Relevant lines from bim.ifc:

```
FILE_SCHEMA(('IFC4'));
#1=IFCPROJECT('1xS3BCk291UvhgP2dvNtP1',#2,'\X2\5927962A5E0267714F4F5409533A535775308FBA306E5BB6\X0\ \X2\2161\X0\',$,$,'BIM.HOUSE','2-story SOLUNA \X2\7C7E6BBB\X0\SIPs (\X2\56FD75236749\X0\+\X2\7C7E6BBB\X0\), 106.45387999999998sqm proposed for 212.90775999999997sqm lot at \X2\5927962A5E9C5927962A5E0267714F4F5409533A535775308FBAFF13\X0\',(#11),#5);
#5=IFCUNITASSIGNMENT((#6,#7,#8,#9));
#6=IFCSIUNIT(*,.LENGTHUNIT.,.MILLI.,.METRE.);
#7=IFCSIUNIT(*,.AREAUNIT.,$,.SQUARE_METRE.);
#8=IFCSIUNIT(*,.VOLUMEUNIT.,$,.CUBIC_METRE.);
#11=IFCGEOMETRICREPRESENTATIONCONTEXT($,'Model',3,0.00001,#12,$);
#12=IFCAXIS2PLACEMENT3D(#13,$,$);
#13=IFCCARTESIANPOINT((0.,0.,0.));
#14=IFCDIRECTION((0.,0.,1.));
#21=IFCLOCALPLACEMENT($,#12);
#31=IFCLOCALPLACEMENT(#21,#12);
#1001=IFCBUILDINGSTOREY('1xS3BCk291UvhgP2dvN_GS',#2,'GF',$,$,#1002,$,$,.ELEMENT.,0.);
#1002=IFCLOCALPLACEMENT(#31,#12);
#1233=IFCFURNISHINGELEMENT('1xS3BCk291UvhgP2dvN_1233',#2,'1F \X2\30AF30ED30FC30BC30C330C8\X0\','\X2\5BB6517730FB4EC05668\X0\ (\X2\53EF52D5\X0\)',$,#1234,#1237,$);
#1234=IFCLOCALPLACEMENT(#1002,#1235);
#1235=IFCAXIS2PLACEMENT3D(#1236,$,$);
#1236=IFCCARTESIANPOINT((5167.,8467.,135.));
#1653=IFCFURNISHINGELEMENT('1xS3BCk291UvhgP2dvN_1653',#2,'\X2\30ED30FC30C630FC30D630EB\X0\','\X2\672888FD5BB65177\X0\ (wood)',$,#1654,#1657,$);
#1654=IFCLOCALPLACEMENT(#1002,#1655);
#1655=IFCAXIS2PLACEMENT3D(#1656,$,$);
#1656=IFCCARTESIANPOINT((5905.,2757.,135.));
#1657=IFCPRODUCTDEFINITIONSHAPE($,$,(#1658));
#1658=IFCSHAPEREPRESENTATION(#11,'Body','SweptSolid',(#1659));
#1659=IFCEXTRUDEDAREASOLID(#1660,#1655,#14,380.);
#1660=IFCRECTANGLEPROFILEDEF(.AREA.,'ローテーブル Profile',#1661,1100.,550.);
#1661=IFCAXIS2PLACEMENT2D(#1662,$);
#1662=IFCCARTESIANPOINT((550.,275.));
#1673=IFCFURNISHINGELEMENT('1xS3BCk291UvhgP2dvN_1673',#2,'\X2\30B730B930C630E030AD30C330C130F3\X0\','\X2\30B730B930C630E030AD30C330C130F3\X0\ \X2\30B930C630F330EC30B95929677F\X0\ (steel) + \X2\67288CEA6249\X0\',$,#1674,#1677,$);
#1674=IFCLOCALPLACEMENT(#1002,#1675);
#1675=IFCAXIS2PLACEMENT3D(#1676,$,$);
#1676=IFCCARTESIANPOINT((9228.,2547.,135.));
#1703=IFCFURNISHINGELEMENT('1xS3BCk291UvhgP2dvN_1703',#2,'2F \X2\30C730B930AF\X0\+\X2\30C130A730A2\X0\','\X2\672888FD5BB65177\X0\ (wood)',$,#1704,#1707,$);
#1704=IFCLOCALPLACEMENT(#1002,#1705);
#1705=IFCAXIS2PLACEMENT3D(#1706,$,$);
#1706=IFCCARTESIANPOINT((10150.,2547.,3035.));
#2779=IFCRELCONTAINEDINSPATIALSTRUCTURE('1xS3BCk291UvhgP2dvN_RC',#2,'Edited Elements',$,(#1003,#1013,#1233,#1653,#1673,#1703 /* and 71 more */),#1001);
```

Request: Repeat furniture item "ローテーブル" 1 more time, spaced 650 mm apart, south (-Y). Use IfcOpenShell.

```python
import numpy as np
import ifcopenshell
import ifcopenshell.api.geometry
import ifcopenshell.api.root
import ifcopenshell.util.element
import ifcopenshell.util.placement
import ifcopenshell.util.unit

model = ifcopenshell.open("bim.ifc")
unit_scale = ifcopenshell.util.unit.calculate_unit_scale(model)


def reuse_history(source, copy):
    """copy_class also copies each property set's owner history, people and application; keep the originals."""
    for rel in copy.IsDefinedBy:
        if rel.is_a("IfcRelDefinesByProperties") and (history := rel.RelatingPropertyDefinition.OwnerHistory):
            rel.RelatingPropertyDefinition.OwnerHistory = source.OwnerHistory
            ifcopenshell.util.element.remove_deep2(model, history)


source = model.by_guid("1xS3BCk291UvhgP2dvN_1653")
base = ifcopenshell.util.placement.get_local_placement(source.ObjectPlacement)
step = np.array([0.0, -1.0, 0.0]) * 0.65 / unit_scale

for i in range(1, 2):
    copy = ifcopenshell.api.root.copy_class(model, product=source)
    copy.Representation = ifcopenshell.util.element.copy_deep(
        model, source.Representation, exclude=["IfcGeometricRepresentationContext", "IfcRepresentationMap"]
    )
    reuse_history(source, copy)
    matrix = base.copy()
    matrix[:3, 3] += i * step
    print("added at", matrix[:3, 3].round(3) + 0.0)
    ifcopenshell.api.geometry.edit_object_placement(model, product=copy, matrix=matrix, is_si=False)

model.write("bim_updated.ifc")
```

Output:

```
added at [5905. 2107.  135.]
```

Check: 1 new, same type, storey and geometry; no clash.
